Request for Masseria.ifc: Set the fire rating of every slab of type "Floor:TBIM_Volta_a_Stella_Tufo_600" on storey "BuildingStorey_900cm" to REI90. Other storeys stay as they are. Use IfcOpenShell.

First a look at what the model holds.

```python
import ifcopenshell
import ifcopenshell.util.element

model = ifcopenshell.open("Masseria.ifc")
print(model.schema)
storey = next(s for s in model.by_type("IfcBuildingStorey") if s.Name == "BuildingStorey_900cm")
slabs = [e for e in ifcopenshell.util.element.get_decomposition(storey) if e.is_a("IfcSlab")]
seen = {}
for e in slabs:
    element_type = ifcopenshell.util.element.get_type(e)
    key = (element_type.Name if element_type != e and element_type else None, ifcopenshell.util.element.get_pset(e, "Pset_SlabCommon", "FireRating"))
    seen[key] = seen.get(key, 0) + 1
for (name, value), count in sorted(seen.items(), key=str):
    print(count, "x", name, "|", value)
```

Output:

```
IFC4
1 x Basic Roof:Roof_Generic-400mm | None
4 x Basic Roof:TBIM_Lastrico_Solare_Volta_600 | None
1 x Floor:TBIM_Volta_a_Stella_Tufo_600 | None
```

```python
import ifcopenshell
import ifcopenshell.api.pset
import ifcopenshell.util.element

model = ifcopenshell.open("Masseria.ifc")

storey = next(s for s in model.by_type("IfcBuildingStorey") if s.Name == "BuildingStorey_900cm")
slabs = [e for e in ifcopenshell.util.element.get_decomposition(storey) if e.is_a("IfcSlab")]

count = 0
for e in slabs:
    element_type = ifcopenshell.util.element.get_type(e)
    if element_type in (None, e) or element_type.Name != "Floor:TBIM_Volta_a_Stella_Tufo_600":
        continue
    # add_pset returns the element's existing set when there is one.
    pset = ifcopenshell.api.pset.add_pset(model, product=e, name="Pset_SlabCommon")
    ifcopenshell.api.pset.edit_pset(model, pset=pset, properties={"FireRating": "REI90"})
    count += 1

print(count, "slabs updated")

model.write("Masseria_edited.ifc")
```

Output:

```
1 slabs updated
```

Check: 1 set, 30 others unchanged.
